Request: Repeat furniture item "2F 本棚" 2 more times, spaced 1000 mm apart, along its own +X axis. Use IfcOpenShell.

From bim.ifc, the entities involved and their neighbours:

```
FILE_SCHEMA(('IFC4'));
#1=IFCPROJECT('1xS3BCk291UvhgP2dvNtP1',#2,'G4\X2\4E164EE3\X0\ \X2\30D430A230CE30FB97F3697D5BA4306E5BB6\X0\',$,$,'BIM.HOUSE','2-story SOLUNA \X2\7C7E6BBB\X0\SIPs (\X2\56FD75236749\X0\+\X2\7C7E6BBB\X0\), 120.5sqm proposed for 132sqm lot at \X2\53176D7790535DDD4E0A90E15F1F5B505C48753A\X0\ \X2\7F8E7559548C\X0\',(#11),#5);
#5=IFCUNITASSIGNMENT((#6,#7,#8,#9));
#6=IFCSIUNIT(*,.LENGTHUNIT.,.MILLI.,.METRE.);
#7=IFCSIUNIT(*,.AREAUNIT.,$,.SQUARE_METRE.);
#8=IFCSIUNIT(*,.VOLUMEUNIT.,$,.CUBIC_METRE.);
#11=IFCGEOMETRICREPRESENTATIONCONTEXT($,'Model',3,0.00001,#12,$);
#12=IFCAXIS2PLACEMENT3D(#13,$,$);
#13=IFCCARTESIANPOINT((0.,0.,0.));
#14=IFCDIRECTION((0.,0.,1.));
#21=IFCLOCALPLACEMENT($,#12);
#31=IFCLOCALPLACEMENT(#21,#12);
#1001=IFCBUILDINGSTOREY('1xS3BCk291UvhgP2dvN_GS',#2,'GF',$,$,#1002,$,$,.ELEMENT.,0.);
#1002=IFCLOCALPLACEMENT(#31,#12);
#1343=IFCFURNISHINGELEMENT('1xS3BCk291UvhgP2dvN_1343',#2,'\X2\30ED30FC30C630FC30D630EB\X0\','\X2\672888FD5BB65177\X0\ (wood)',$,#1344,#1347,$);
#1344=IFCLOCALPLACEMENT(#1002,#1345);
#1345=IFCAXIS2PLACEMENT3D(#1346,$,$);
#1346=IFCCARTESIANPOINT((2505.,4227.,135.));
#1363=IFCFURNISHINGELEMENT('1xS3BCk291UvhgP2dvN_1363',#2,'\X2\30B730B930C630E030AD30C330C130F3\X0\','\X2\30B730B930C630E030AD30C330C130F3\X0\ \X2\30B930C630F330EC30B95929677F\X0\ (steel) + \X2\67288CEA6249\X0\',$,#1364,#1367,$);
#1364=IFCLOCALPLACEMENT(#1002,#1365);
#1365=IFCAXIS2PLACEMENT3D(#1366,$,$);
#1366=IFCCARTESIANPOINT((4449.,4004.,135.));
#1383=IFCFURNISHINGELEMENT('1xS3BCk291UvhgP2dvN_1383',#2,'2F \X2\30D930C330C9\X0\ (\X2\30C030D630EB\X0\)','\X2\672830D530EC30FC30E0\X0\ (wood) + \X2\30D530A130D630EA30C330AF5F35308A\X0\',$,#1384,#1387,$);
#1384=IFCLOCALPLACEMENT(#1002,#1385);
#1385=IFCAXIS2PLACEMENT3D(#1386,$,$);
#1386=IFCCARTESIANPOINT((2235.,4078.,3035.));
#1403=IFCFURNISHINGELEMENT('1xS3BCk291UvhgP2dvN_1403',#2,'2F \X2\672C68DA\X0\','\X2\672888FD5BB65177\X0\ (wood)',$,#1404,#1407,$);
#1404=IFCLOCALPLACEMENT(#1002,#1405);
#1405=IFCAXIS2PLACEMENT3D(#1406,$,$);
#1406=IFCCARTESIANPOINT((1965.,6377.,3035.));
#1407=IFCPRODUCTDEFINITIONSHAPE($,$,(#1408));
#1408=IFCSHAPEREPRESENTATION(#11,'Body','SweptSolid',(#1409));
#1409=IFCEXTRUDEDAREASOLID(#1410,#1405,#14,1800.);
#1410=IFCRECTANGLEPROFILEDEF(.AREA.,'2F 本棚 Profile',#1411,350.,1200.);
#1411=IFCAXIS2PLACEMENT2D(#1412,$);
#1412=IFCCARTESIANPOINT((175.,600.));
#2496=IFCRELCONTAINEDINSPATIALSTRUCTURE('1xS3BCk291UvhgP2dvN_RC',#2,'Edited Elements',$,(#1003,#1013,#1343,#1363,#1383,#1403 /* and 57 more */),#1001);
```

```python
import ifcopenshell
import ifcopenshell.api.geometry
import ifcopenshell.api.root
import ifcopenshell.util.element
import ifcopenshell.util.placement
import ifcopenshell.util.unit

model = ifcopenshell.open("bim.ifc")
unit_scale = ifcopenshell.util.unit.calculate_unit_scale(model)


def reuse_history(source, copy):
    """copy_class also copies each property set's owner history, people and application; keep the originals."""
    for rel in copy.IsDefinedBy:
        if rel.is_a("IfcRelDefinesByProperties") and (history := rel.RelatingPropertyDefinition.OwnerHistory):
            rel.RelatingPropertyDefinition.OwnerHistory = source.OwnerHistory
            ifcopenshell.util.element.remove_deep2(model, history)


source = model.by_id(1403)
base = ifcopenshell.util.placement.get_local_placement(source.ObjectPlacement)
step = base[:3, 0] * 1 / unit_scale

for i in range(1, 3):
    copy = ifcopenshell.api.root.copy_class(model, product=source)
    copy.Representation = ifcopenshell.util.element.copy_deep(
        model, source.Representation, exclude=["IfcGeometricRepresentationContext", "IfcRepresentationMap"]
    )
    reuse_history(source, copy)
    matrix = base.copy()
    matrix[:3, 3] += i * step
    print("added at", matrix[:3, 3].round(3) + 0.0)
    ifcopenshell.api.geometry.edit_object_placement(model, product=copy, matrix=matrix, is_si=False)

model.write("bim_updated.ifc")
```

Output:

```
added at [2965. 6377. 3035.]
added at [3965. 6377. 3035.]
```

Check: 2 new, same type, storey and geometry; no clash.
